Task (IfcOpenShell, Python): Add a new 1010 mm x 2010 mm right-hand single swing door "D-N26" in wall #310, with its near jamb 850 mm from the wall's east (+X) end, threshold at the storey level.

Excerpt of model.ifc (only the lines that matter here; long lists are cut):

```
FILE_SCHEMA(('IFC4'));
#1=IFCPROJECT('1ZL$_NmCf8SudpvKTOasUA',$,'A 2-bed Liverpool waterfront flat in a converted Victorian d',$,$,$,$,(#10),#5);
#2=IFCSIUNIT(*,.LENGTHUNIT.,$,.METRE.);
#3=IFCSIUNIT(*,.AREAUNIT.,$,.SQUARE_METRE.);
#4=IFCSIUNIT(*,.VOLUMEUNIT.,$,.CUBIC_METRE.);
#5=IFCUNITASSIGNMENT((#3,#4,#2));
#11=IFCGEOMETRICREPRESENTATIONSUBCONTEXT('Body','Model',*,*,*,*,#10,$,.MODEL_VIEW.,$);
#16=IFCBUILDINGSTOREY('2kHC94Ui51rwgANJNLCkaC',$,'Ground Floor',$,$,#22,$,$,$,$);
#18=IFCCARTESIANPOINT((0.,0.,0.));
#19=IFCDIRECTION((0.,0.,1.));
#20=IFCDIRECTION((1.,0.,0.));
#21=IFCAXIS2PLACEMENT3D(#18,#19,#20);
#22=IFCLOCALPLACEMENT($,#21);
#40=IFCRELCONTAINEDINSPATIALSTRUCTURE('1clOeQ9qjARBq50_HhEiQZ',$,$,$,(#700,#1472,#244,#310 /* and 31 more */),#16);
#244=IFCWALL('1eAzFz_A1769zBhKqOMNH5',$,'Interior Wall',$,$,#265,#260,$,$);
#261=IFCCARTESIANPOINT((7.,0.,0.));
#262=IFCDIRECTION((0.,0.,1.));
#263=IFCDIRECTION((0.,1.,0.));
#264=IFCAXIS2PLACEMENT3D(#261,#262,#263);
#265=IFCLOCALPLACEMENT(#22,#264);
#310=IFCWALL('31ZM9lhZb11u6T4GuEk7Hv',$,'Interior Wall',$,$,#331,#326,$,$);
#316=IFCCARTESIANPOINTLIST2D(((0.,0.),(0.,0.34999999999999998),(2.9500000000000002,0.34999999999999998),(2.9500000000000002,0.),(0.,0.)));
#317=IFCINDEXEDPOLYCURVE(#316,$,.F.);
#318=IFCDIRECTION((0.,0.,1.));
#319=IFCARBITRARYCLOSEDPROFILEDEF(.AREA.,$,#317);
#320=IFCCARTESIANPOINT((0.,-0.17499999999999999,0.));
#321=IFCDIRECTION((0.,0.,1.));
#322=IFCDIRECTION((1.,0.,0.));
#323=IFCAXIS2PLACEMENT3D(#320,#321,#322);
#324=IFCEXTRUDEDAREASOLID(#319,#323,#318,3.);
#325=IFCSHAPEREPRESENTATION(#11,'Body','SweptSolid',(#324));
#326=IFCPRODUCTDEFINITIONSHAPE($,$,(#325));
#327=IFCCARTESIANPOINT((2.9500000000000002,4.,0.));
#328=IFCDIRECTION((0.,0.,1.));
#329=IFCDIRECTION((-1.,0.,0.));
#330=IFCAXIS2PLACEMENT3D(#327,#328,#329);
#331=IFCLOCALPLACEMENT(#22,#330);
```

```python
import numpy as np
import ifcopenshell
import ifcopenshell.api.feature
import ifcopenshell.api.geometry
import ifcopenshell.api.root
import ifcopenshell.api.spatial
import ifcopenshell.geom
import ifcopenshell.util.element
import ifcopenshell.util.placement
import ifcopenshell.util.representation
import ifcopenshell.util.shape
import ifcopenshell.util.unit

model = ifcopenshell.open("model.ifc")
unit_scale = ifcopenshell.util.unit.calculate_unit_scale(model)
settings = ifcopenshell.geom.settings()


def volume(element):
    """Net volume in cubic metres, openings subtracted."""
    shape = ifcopenshell.geom.create_shape(settings, element)
    return ifcopenshell.util.shape.get_volume(shape.geometry)


wall = model.by_guid("31ZM9lhZb11u6T4GuEk7Hv")
storey = ifcopenshell.util.element.get_container(wall, ifc_class="IfcBuildingStorey")
context = ifcopenshell.util.representation.get_context(model, "Model", "Body", "MODEL_VIEW")
before = volume(wall)

width, height, from_end, sill = 1.01, 2.01, 0.85, 0.0  # metres

# The wall runs along its own X axis, and the end named is its -X end.
wall_shape = ifcopenshell.geom.create_shape(settings, wall)
x, y, z = ifcopenshell.util.shape.get_vertices(wall_shape.geometry).T
start = x.min() + from_end
face, thickness = float(y.min()), float(y.max() - y.min())
wall_matrix = ifcopenshell.util.placement.get_local_placement(wall.ObjectPlacement)
level = ifcopenshell.util.placement.get_local_placement(storey.ObjectPlacement)[2, 3]


def in_wall(x, y):
    """Placement at x, y metres in the wall's axes, at sill height."""
    matrix = wall_matrix.copy()
    matrix[:, 3] = wall_matrix @ np.array([x / unit_scale, y / unit_scale, 0.0, 1.0])
    matrix[2, 3] = level + sill / unit_scale
    return matrix


# Opening: a box that overshoots both wall faces by 50 mm.
opening = ifcopenshell.api.root.create_entity(model, ifc_class="IfcOpeningElement", predefined_type="OPENING")
box = ifcopenshell.api.geometry.add_wall_representation(
    model, context=context, length=width, height=height, thickness=thickness + 0.1
)
ifcopenshell.api.geometry.assign_representation(model, product=opening, representation=box)
ifcopenshell.api.geometry.edit_object_placement(model, product=opening, matrix=in_wall(start, face - 0.05), is_si=False)
ifcopenshell.api.feature.add_feature(model, feature=opening, element=wall)

door = ifcopenshell.api.root.create_entity(model, ifc_class="IfcDoor", name="D-N26", predefined_type="DOOR")
door.OverallWidth, door.OverallHeight = width / unit_scale, height / unit_scale
door.OperationType = "SINGLE_SWING_RIGHT"
body = ifcopenshell.api.geometry.add_door_representation(
    model,
    context=context,
    overall_width=door.OverallWidth,
    overall_height=door.OverallHeight,
    operation_type="SINGLE_SWING_RIGHT",
    lining_properties={"LiningDepth": thickness / unit_scale, "ThresholdDepth": thickness / unit_scale},
)
ifcopenshell.api.geometry.assign_representation(model, product=door, representation=body)
ifcopenshell.api.spatial.assign_container(model, products=[door], relating_structure=storey)
ifcopenshell.api.feature.add_filling(model, opening=opening, element=door)

# The lining spans the wall, so the door starts at the wall face.
ifcopenshell.api.geometry.edit_object_placement(model, product=door, matrix=in_wall(start, face), is_si=False)

after = volume(wall)

print(f"wall volume {before:.3f} -> {after:.3f} m3")

model.write("model_rev.ifc")
```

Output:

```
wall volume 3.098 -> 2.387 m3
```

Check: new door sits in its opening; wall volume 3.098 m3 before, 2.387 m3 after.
